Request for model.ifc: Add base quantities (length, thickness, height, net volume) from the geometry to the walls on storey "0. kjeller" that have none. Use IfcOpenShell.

First a look at what the model holds.

```python
import ifcopenshell
import ifcopenshell.util.element
import ifcopenshell.util.unit

model = ifcopenshell.open("model.ifc")
print(model.schema)
for unit_type in ("LENGTHUNIT", "AREAUNIT", "VOLUMEUNIT"):
    print(unit_type, ifcopenshell.util.unit.calculate_unit_scale(model, unit_type))
storey = next(s for s in model.by_type("IfcBuildingStorey") if s.Name == "0. kjeller")
walls = [e for e in ifcopenshell.util.element.get_decomposition(storey) if e.is_a("IfcWall")]
for e in sorted(walls, key=lambda e: e.id()):
    print(e.id(), e.is_a(), e.Name, list(ifcopenshell.util.element.get_psets(e, qtos_only=True)), sep=" | ")
```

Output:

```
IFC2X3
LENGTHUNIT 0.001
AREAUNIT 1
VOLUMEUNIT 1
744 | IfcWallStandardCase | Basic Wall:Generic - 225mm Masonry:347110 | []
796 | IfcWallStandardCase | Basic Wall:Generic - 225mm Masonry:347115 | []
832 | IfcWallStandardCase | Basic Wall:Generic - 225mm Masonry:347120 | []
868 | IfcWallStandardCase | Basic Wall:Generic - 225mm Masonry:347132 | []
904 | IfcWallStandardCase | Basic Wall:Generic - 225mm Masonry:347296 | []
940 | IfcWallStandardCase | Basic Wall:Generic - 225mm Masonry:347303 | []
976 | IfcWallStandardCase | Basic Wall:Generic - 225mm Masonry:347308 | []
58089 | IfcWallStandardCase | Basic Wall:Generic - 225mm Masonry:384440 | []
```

```python
import ifcopenshell
import ifcopenshell.api.pset
import ifcopenshell.geom
import ifcopenshell.util.element
import ifcopenshell.util.shape
import ifcopenshell.util.unit

model = ifcopenshell.open("model.ifc")
unit_scale = ifcopenshell.util.unit.calculate_unit_scale(model)
volume_scale = ifcopenshell.util.unit.calculate_unit_scale(model, "VOLUMEUNIT")
settings = ifcopenshell.geom.settings()

storey = next(s for s in model.by_type("IfcBuildingStorey") if s.Name == "0. kjeller")
walls = [e for e in ifcopenshell.util.element.get_decomposition(storey) if e.is_a("IfcWall")]

for e in sorted(walls, key=lambda e: e.id()):
    if ifcopenshell.util.element.get_psets(e, qtos_only=True, should_inherit=False):
        continue
    # Geometry comes back in metres, in the element's own axes.
    shape = ifcopenshell.geom.create_shape(settings, e)
    values = {
        "Length": ifcopenshell.util.shape.get_x(shape.geometry) / unit_scale,
        "Width": ifcopenshell.util.shape.get_y(shape.geometry) / unit_scale,
        "Height": ifcopenshell.util.shape.get_z(shape.geometry) / unit_scale,
        "NetVolume": ifcopenshell.util.shape.get_volume(shape.geometry) / volume_scale,
    }
    qto = ifcopenshell.api.pset.add_qto(model, product=e, name="BaseQuantities")
    ifcopenshell.api.pset.edit_qto(model, qto=qto, properties=values)
    print(e.id(), {k: round(v, 3) for k, v in values.items()})

model.write("model_updated.ifc")
```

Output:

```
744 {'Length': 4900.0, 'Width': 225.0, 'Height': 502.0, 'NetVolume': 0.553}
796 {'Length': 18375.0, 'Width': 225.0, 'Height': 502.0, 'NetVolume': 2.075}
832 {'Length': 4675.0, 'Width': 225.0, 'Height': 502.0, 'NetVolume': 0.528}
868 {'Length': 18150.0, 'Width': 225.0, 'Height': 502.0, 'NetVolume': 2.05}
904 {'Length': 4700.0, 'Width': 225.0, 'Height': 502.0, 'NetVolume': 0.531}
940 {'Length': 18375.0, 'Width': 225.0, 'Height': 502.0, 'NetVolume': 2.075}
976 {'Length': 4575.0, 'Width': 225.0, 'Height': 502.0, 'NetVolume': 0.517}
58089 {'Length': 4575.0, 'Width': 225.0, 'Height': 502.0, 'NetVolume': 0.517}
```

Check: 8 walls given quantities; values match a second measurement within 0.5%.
